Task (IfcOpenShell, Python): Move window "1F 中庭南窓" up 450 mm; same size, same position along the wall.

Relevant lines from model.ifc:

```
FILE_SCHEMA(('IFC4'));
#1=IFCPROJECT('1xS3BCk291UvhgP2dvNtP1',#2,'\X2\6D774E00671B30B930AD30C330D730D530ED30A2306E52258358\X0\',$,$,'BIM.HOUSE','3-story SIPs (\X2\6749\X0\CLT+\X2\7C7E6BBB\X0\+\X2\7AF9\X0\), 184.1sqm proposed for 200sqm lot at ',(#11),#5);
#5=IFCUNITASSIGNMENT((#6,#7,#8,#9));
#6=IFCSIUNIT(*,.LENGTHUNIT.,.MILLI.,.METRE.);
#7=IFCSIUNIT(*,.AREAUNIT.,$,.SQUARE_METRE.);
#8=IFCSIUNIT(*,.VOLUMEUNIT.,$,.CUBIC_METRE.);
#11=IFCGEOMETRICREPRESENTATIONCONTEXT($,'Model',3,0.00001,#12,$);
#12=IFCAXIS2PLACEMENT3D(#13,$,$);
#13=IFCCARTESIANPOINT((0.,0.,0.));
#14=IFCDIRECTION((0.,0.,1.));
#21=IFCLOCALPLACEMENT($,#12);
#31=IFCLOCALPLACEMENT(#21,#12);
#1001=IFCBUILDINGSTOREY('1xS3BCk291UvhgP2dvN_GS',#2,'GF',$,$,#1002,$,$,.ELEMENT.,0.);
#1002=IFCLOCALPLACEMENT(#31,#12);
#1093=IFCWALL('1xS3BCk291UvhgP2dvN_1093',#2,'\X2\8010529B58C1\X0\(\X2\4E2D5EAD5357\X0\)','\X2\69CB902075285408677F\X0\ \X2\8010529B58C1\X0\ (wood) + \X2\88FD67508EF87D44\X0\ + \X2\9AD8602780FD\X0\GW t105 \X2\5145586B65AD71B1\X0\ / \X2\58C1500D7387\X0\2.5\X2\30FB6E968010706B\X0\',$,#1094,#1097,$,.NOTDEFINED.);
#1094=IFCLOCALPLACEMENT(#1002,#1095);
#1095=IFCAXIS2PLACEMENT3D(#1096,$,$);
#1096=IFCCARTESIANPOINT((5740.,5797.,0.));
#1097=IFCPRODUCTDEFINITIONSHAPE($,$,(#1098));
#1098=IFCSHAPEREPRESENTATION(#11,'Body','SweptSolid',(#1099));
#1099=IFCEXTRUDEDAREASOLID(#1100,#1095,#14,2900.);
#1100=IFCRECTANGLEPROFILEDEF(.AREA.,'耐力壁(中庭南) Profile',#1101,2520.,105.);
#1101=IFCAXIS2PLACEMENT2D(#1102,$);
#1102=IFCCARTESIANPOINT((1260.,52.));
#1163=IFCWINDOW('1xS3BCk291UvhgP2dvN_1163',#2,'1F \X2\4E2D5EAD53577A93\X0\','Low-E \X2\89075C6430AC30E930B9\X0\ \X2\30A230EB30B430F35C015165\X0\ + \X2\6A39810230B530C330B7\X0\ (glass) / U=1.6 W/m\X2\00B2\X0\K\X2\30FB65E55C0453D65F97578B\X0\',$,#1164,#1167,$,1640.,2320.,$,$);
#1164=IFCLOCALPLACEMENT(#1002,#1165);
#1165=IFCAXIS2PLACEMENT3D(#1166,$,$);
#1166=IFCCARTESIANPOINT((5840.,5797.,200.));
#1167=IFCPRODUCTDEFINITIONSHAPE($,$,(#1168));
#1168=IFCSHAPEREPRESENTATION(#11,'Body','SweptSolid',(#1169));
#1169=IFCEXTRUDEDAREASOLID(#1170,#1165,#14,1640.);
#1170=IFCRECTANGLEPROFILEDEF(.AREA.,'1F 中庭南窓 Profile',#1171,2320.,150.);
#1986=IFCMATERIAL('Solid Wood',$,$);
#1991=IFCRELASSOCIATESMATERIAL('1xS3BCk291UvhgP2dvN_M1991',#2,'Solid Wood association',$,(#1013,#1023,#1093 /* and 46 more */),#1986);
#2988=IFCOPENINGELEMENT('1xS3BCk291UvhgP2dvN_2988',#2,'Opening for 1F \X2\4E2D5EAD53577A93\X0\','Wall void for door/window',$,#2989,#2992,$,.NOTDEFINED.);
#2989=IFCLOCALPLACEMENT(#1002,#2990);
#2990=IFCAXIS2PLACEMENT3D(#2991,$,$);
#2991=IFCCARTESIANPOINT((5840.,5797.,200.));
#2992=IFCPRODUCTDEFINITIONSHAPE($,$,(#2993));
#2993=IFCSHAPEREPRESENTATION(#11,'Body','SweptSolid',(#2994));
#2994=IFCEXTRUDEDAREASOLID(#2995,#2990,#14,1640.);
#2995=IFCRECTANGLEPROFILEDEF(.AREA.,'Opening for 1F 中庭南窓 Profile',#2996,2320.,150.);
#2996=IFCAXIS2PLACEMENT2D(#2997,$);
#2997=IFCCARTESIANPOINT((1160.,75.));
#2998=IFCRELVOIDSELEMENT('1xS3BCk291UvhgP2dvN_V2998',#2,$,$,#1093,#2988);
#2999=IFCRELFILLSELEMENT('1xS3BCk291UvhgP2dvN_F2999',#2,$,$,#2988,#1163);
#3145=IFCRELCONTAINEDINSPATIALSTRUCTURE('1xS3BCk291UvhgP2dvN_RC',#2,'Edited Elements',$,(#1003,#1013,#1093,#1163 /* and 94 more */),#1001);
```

```python
import numpy as np
import ifcopenshell
import ifcopenshell.api.geometry
import ifcopenshell.util.placement
import ifcopenshell.util.unit

model = ifcopenshell.open("model.ifc")
unit_scale = ifcopenshell.util.unit.calculate_unit_scale(model)

window = model.by_guid("1xS3BCk291UvhgP2dvN_1163")
opening = window.FillsVoids[0].RelatingOpeningElement
dz = 0.45 / unit_scale

shift = np.array([0.0, 0.0, dz])
# The window is not placed relative to its opening, so move both.
for product in (opening, window):
    matrix = ifcopenshell.util.placement.get_local_placement(product.ObjectPlacement)
    matrix[:3, 3] += shift
    ifcopenshell.api.geometry.edit_object_placement(model, product=product, matrix=matrix, is_si=False)

print(f"moved by {dz * unit_scale:+.3f} m")

model.write("model_rev.ifc")
```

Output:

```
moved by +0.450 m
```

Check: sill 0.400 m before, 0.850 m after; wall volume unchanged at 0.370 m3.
